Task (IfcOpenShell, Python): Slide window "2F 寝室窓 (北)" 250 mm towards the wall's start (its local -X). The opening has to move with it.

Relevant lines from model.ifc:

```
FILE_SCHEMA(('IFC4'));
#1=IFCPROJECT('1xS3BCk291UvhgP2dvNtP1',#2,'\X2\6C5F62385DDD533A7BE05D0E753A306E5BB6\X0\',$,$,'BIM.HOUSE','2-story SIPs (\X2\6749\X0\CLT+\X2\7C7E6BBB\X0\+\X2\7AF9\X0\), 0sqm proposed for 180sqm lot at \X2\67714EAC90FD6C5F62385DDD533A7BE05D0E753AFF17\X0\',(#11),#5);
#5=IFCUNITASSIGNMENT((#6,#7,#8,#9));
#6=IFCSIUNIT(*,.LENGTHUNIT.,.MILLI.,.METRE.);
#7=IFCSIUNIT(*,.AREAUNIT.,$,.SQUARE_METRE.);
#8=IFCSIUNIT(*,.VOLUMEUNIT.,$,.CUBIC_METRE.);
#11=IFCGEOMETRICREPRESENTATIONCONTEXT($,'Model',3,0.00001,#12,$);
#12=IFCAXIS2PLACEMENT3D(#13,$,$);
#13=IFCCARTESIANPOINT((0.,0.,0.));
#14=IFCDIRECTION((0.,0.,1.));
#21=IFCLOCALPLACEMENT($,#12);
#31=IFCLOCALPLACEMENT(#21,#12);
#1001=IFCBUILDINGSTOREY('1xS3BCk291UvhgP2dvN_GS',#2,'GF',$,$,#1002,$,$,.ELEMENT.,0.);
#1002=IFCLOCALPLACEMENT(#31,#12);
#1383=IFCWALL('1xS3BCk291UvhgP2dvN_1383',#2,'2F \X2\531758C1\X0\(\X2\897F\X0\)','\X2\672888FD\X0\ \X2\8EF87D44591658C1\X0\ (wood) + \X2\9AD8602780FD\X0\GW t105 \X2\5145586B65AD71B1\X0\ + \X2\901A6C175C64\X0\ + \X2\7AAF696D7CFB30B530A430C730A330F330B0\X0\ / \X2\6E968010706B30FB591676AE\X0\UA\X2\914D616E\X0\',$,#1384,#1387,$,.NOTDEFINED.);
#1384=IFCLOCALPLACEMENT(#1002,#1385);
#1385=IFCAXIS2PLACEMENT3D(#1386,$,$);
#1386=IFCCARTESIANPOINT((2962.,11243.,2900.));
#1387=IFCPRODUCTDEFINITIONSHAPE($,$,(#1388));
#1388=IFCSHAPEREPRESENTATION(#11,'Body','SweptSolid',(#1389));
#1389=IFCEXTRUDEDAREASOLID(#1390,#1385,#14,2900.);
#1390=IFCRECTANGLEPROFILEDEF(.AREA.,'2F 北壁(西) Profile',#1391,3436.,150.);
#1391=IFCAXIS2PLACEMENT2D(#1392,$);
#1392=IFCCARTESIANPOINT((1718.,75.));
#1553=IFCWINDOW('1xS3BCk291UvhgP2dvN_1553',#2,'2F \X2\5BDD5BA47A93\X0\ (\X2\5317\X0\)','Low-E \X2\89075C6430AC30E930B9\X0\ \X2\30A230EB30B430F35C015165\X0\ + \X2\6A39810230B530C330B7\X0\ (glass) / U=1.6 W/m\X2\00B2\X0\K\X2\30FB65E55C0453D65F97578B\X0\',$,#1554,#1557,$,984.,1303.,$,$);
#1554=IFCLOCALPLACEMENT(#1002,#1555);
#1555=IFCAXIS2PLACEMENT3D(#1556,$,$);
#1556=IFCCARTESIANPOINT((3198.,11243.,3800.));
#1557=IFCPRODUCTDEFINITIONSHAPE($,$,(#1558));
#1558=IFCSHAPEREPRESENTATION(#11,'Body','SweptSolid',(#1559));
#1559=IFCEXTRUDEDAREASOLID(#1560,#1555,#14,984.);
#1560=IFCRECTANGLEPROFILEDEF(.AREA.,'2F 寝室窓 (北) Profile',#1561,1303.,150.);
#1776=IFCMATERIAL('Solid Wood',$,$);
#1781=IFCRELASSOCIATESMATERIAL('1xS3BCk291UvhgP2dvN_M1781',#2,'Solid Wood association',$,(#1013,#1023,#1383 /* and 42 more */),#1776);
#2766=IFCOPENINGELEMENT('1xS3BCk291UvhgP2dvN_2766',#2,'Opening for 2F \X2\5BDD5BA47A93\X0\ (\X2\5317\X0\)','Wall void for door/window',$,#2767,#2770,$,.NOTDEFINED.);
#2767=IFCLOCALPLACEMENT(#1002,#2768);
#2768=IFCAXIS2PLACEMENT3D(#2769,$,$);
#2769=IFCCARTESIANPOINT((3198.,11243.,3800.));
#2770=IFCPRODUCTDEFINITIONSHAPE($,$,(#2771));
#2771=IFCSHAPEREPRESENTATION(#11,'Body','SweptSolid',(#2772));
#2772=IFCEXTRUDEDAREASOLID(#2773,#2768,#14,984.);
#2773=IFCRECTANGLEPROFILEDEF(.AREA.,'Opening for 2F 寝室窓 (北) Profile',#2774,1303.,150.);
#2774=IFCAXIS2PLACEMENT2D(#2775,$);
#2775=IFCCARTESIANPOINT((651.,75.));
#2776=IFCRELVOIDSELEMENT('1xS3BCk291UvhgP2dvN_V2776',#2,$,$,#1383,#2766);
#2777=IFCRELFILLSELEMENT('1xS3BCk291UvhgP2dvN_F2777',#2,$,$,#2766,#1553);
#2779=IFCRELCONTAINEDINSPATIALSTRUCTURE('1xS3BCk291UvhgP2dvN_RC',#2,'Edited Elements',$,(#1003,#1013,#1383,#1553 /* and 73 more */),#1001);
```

```python
import ifcopenshell
import ifcopenshell.api.geometry
import ifcopenshell.util.placement
import ifcopenshell.util.unit

model = ifcopenshell.open("model.ifc")
unit_scale = ifcopenshell.util.unit.calculate_unit_scale(model)

window = model.by_guid("1xS3BCk291UvhgP2dvN_1553")
opening = window.FillsVoids[0].RelatingOpeningElement
wall = opening.VoidsElements[0].RelatingBuildingElement

wall_matrix = ifcopenshell.util.placement.get_local_placement(wall.ObjectPlacement)
shift = wall_matrix[:3, 0] * -0.25 / unit_scale
before = ifcopenshell.util.placement.get_local_placement(window.ObjectPlacement)[:3, 3].copy()

# The window is not placed relative to its opening, so move both.
for product in (opening, window):
    matrix = ifcopenshell.util.placement.get_local_placement(product.ObjectPlacement)
    matrix[:3, 3] += shift
    ifcopenshell.api.geometry.edit_object_placement(model, product=product, matrix=matrix, is_si=False)

after = ifcopenshell.util.placement.get_local_placement(window.ObjectPlacement)[:3, 3]
print("window moved by", (after - before).round(3) + 0.0)

model.write("model_v2.ifc")
```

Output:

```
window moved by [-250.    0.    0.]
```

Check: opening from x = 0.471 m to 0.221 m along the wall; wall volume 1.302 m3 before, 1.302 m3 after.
